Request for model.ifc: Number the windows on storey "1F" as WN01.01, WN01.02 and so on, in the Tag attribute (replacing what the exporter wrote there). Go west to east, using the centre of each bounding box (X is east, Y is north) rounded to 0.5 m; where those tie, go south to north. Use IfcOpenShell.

First a look at what the model holds.

```python
import ifcopenshell
import ifcopenshell.util.element
import ifcopenshell.util.placement

model = ifcopenshell.open("model.ifc")
print(model.schema)
storey = next(s for s in model.by_type("IfcBuildingStorey") if s.Name == "1F")
windows = [e for e in ifcopenshell.util.element.get_decomposition(storey) if e.is_a("IfcWindow")]
for e in sorted(windows, key=lambda e: e.id()):
    origin = ifcopenshell.util.placement.get_local_placement(e.ObjectPlacement)[:3, 3]
    print(e.id(), e.Tag, e.Name, origin.round(2) + 0.0, sep=" | ")
```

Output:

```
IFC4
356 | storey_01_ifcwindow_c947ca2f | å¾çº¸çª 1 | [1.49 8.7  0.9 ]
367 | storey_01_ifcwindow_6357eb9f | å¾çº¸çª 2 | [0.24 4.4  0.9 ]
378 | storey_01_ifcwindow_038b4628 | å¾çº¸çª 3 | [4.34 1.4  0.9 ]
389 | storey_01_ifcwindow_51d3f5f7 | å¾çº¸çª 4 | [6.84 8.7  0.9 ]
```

```python
import ifcopenshell
import ifcopenshell.geom
import ifcopenshell.util.element
import ifcopenshell.util.shape

model = ifcopenshell.open("model.ifc")
settings = ifcopenshell.geom.settings()
settings.set("use-world-coords", True)


def centre(element):
    shape = ifcopenshell.geom.create_shape(settings, element)
    return ifcopenshell.util.shape.get_bbox_centroid(shape.geometry)


storey = next(s for s in model.by_type("IfcBuildingStorey") if s.Name == "1F")
windows = [e for e in ifcopenshell.util.element.get_decomposition(storey) if e.is_a("IfcWindow")]

# Insertion points can sit at a corner or the storey origin, so sort by the geometry (in metres).
centres = {e: centre(e) for e in windows}
windows.sort(key=lambda e: (round(centres[e][0] / 0.5), centres[e][1]))

for i, e in enumerate(windows, start=1):
    number = f"WN01.{i:02d}"
    e.Tag = number
    print(e.id(), number)

model.write("model_updated.ifc")
```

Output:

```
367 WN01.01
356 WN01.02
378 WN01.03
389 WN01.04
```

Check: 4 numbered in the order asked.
